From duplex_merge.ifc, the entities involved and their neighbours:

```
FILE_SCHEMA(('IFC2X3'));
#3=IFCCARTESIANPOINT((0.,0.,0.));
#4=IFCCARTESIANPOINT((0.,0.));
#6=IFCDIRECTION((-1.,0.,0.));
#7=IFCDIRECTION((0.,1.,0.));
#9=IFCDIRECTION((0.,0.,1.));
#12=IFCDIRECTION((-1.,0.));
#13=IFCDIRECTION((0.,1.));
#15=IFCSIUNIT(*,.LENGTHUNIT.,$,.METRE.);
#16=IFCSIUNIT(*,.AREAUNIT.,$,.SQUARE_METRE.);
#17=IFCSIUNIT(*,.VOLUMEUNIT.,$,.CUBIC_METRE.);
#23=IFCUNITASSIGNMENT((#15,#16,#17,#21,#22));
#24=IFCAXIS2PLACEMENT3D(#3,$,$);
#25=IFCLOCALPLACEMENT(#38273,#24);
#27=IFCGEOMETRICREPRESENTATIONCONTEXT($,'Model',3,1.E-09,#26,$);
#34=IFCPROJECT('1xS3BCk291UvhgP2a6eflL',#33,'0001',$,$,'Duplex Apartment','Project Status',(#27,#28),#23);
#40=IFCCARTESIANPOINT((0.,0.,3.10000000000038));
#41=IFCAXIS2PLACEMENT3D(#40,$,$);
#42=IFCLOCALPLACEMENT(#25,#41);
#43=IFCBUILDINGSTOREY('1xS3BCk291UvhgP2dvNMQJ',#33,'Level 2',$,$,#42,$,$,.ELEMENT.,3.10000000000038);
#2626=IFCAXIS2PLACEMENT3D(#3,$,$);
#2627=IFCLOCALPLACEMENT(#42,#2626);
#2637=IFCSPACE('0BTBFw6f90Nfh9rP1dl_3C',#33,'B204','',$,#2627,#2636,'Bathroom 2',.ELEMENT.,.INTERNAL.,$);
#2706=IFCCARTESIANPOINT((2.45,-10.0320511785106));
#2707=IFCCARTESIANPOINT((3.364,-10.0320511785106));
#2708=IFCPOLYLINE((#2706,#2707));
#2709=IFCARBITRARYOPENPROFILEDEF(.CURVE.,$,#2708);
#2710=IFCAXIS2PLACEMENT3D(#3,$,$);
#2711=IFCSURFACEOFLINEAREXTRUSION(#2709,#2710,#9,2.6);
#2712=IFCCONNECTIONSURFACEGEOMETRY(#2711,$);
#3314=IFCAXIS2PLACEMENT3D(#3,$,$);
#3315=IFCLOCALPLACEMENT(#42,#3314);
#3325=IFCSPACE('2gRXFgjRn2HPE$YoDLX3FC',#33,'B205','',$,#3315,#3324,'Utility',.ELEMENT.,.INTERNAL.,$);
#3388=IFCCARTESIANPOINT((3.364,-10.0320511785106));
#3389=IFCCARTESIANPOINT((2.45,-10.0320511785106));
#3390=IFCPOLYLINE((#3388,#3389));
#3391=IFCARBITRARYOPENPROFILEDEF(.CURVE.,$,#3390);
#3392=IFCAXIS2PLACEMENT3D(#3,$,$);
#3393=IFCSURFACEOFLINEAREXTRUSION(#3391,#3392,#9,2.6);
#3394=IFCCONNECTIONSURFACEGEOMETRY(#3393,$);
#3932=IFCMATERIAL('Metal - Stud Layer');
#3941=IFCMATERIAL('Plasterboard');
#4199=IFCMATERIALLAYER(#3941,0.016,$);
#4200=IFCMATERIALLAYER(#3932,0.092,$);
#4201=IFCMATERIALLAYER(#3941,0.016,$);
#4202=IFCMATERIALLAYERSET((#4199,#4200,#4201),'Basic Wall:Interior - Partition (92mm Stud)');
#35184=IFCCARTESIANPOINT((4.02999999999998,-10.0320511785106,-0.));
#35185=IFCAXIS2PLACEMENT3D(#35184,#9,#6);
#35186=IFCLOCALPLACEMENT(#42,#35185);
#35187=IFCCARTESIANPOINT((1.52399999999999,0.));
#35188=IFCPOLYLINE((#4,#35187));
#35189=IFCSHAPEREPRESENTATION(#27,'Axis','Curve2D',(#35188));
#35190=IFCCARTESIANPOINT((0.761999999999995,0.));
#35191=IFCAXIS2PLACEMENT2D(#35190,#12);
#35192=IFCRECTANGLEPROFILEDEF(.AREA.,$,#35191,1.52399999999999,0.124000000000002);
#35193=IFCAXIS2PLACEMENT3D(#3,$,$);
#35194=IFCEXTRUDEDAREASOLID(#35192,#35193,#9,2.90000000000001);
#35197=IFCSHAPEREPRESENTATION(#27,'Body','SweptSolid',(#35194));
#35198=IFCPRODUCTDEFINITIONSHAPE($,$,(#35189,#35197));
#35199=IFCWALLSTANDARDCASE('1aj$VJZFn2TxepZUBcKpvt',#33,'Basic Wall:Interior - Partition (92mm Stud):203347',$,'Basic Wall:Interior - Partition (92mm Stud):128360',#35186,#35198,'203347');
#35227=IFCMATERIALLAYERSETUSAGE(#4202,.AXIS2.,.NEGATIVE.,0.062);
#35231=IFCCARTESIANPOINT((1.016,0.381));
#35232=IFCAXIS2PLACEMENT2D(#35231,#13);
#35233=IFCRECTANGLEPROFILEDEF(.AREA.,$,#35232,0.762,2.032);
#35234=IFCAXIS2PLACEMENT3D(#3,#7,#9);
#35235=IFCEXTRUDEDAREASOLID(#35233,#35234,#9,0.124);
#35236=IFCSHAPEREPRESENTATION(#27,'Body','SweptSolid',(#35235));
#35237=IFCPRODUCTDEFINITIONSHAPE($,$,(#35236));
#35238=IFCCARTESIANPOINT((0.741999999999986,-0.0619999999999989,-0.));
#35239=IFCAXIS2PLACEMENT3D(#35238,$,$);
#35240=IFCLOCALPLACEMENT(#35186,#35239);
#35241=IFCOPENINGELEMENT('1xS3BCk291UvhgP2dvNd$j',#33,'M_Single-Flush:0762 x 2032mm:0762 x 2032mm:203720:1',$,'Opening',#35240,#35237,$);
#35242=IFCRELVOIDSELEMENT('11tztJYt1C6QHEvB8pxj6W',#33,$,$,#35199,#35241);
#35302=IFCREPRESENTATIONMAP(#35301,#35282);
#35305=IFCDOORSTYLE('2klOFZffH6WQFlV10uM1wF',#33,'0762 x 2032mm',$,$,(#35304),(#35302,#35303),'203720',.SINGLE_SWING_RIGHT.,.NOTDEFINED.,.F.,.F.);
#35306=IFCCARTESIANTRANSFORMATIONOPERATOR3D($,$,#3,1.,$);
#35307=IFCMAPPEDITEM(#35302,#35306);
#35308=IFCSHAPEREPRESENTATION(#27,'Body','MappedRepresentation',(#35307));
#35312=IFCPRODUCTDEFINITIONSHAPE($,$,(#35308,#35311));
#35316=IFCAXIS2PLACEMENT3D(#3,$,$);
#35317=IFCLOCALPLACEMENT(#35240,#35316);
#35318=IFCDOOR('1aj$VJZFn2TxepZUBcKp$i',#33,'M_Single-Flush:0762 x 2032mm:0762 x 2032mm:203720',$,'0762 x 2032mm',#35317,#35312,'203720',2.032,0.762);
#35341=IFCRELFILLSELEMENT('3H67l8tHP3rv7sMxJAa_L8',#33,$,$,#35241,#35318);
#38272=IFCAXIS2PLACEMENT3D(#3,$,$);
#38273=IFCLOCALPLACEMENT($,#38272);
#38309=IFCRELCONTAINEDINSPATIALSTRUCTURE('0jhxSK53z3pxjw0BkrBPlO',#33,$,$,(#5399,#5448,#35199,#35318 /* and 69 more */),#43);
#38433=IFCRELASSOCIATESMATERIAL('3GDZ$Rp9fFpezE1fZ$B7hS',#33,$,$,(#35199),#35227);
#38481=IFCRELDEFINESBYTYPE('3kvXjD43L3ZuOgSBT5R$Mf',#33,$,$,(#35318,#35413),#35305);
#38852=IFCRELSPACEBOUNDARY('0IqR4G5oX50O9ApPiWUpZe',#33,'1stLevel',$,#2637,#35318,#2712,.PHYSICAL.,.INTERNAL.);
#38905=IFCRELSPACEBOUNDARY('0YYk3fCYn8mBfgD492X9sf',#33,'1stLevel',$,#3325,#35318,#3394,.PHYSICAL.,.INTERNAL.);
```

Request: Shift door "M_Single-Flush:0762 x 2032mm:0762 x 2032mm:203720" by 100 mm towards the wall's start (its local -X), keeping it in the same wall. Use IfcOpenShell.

```python
import numpy as np
import ifcopenshell
import ifcopenshell.api.geometry
import ifcopenshell.util.placement

model = ifcopenshell.open("duplex_merge.ifc")

door = model.by_id(35318)
opening = door.FillsVoids[0].RelatingOpeningElement
wall = opening.VoidsElements[0].RelatingBuildingElement

wall_matrix = ifcopenshell.util.placement.get_local_placement(wall.ObjectPlacement)
shift = wall_matrix[:3, 0] * -0.1
before = ifcopenshell.util.placement.get_local_placement(door.ObjectPlacement)[:3, 3].copy()

# The door is placed relative to its opening, so it follows when the opening moves.
matrix = ifcopenshell.util.placement.get_local_placement(opening.ObjectPlacement)
matrix[:3, 3] += shift
ifcopenshell.api.geometry.edit_object_placement(
    model, product=opening, matrix=matrix, is_si=False, should_transform_children=True
)

# Space boundary surfaces are stored in each space's coordinates; move them too.
for rel in door.ProvidesBoundaries:
    if not rel.ConnectionGeometry:
        continue
    surface = rel.ConnectionGeometry.SurfaceOnRelatingElement
    space_matrix = ifcopenshell.util.placement.get_local_placement(rel.RelatingSpace.ObjectPlacement)
    point = np.array(surface.Position.Location.Coordinates) + space_matrix[:3, :3].T @ shift
    surface.Position = model.createIfcAxis2Placement3D(
        model.createIfcCartesianPoint(point.tolist()), surface.Position.Axis, surface.Position.RefDirection
    )

after = ifcopenshell.util.placement.get_local_placement(door.ObjectPlacement)[:3, 3]
print("door moved by", (after - before).round(3) + 0.0)

model.write("duplex_merge_v2.ifc")
```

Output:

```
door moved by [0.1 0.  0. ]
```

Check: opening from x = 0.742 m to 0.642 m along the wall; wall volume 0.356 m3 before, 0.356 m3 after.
